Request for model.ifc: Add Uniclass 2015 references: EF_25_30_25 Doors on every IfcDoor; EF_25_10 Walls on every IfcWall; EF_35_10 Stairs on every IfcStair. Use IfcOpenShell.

First a look at what the model holds.

```python
import ifcopenshell

model = ifcopenshell.open("model.ifc")
print(model.schema)
print("classifications:", [c.Name for c in model.by_type("IfcClassification")])
for ifc_class in ("IfcDoor", "IfcRoof", "IfcStair", "IfcWall", "IfcWindow"):
    print(ifc_class, len(model.by_type(ifc_class)))
```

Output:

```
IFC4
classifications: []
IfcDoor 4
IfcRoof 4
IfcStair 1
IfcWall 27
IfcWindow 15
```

```python
import ifcopenshell
import ifcopenshell.api.classification

model = ifcopenshell.open("model.ifc")

system = ifcopenshell.api.classification.add_classification(model, classification="Uniclass 2015")

codes = {
    "IfcDoor": ("EF_25_30_25", "Doors"),
    "IfcWall": ("EF_25_10", "Walls"),
    "IfcStair": ("EF_35_10", "Stairs"),
}
for ifc_class, (code, name) in codes.items():
    products = model.by_type(ifc_class)
    ifcopenshell.api.classification.add_reference(
        model, products=products, classification=system, identification=code, name=name
    )
    print(code, len(products))

model.write("model_edited.ifc")
```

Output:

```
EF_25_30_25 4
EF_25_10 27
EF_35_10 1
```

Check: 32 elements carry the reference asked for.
